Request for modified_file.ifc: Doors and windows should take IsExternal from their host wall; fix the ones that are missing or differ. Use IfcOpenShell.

First a look at what the model holds.

```python
import ifcopenshell
import ifcopenshell.util.element

model = ifcopenshell.open("modified_file.ifc")
print(model.schema)
seen = {}
for e in model.by_type("IfcDoor") + model.by_type("IfcWindow"):
    if not e.FillsVoids:
        continue
    host = e.FillsVoids[0].RelatingOpeningElement.VoidsElements[0].RelatingBuildingElement
    own = ifcopenshell.util.element.get_pset(e, f"Pset_{e.is_a()[3:].removesuffix('StandardCase')}Common", "IsExternal")
    wall = ifcopenshell.util.element.get_pset(host, "Pset_WallCommon", "IsExternal")
    seen[e.is_a(), own, wall] = seen.get((e.is_a(), own, wall), 0) + 1
for (cls, own, wall), count in sorted(seen.items(), key=str):
    print(count, cls, "IsExternal:", own, "| host wall:", wall)
```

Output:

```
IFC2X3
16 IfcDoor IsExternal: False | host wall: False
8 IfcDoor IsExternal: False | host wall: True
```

```python
import ifcopenshell
import ifcopenshell.api.pset
import ifcopenshell.util.element

model = ifcopenshell.open("modified_file.ifc")

count = 0
for ifc_class, pset_name in (("IfcDoor", "Pset_DoorCommon"), ("IfcWindow", "Pset_WindowCommon")):
    for e in model.by_type(ifc_class):
        if not e.FillsVoids:
            continue
        host = e.FillsVoids[0].RelatingOpeningElement.VoidsElements[0].RelatingBuildingElement
        external = ifcopenshell.util.element.get_pset(host, "Pset_WallCommon", "IsExternal")
        if external is None or ifcopenshell.util.element.get_pset(e, pset_name, "IsExternal") == external:
            continue
        pset = ifcopenshell.api.pset.add_pset(model, product=e, name=pset_name)
        ifcopenshell.api.pset.edit_pset(model, pset=pset, properties={"IsExternal": external})
        count += 1

print(count, "updated")

model.write("modified_file_edited.ifc")
```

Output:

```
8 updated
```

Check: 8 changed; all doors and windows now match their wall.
